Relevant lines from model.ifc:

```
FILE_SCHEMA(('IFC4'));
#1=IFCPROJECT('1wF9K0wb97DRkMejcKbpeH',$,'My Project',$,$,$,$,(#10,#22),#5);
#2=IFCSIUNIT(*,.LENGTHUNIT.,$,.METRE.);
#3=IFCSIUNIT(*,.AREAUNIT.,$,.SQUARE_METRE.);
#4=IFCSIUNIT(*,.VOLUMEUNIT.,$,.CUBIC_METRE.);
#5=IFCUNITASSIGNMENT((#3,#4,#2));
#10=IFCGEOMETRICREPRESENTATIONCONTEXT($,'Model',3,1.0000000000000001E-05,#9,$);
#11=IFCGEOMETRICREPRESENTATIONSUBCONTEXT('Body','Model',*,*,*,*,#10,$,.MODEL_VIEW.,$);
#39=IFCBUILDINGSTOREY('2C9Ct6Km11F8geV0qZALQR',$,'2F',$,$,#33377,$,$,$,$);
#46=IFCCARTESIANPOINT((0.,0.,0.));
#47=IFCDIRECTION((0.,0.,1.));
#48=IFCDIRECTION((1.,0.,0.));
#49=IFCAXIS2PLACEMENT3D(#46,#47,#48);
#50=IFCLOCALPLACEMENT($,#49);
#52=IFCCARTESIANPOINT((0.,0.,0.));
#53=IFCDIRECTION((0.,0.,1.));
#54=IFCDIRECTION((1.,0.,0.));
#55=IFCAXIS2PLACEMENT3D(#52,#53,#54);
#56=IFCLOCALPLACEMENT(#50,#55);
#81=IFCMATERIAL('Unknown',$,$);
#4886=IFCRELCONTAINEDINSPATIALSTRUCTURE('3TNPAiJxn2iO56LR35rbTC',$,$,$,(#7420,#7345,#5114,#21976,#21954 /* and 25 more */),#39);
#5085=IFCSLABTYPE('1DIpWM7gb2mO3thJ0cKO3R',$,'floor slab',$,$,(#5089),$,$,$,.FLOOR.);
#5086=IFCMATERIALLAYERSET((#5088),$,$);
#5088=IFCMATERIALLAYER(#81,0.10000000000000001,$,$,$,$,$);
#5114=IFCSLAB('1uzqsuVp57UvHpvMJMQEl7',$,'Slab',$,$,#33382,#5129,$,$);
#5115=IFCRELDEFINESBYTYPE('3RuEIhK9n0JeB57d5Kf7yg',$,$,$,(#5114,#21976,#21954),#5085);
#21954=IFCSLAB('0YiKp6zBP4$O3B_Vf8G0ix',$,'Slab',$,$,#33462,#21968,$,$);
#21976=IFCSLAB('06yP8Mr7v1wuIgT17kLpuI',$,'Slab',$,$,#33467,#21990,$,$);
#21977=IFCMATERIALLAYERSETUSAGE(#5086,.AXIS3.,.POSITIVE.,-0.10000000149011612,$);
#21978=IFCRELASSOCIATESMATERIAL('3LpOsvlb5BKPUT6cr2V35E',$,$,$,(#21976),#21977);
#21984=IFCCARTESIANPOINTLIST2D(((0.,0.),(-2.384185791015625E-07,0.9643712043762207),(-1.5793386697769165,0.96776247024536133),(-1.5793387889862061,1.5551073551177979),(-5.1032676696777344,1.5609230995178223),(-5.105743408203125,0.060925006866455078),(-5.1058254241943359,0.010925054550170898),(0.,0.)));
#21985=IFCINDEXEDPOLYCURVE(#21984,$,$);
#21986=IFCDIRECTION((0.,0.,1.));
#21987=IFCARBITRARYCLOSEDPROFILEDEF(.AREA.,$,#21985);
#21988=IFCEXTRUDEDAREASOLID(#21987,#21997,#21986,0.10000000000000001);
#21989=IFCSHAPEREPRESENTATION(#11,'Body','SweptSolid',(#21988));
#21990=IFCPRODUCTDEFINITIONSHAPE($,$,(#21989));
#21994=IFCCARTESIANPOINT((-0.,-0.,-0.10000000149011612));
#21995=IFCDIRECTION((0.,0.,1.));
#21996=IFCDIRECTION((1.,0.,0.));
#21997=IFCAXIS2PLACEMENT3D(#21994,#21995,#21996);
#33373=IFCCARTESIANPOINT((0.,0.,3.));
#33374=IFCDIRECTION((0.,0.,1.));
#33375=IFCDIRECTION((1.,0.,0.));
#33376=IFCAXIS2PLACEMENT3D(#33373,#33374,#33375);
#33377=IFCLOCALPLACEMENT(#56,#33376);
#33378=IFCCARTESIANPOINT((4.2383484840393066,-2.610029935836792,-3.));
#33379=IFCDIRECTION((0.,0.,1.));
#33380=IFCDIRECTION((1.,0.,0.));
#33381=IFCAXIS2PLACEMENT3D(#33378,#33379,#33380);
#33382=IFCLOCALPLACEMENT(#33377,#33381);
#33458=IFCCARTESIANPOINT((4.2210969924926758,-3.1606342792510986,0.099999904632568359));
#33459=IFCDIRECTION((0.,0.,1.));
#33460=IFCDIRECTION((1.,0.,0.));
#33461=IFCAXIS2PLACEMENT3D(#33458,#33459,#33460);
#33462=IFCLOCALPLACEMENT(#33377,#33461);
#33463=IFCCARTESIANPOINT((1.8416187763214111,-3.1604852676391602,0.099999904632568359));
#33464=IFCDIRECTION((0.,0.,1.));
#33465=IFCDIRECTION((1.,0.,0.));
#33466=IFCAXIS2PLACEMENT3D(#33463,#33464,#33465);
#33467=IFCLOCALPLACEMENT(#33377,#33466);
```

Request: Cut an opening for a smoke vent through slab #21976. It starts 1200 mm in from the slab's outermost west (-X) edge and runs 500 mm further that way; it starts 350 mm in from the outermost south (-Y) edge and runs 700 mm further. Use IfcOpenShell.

```python
import numpy as np
import ifcopenshell
import ifcopenshell.api.feature
import ifcopenshell.api.geometry
import ifcopenshell.api.root
import ifcopenshell.geom
import ifcopenshell.util.placement
import ifcopenshell.util.representation
import ifcopenshell.util.shape
import ifcopenshell.util.unit

model = ifcopenshell.open("model.ifc")
unit_scale = ifcopenshell.util.unit.calculate_unit_scale(model)
settings = ifcopenshell.geom.settings()


def volume(element):
    """Net volume in cubic metres, openings subtracted."""
    shape = ifcopenshell.geom.create_shape(settings, element)
    return ifcopenshell.util.shape.get_volume(shape.geometry)


slab = model.by_guid("06yP8Mr7v1wuIgT17kLpuI")
before = volume(slab)

# Extent in the slab's own axes, in metres. The edges named are its -X and -Y sides.
slab_shape = ifcopenshell.geom.create_shape(settings, slab)
vertices = ifcopenshell.util.shape.get_vertices(slab_shape.geometry)
x_min, y_min, bottom = vertices.min(axis=0)
top = vertices[:, 2].max()

opening = ifcopenshell.api.root.create_entity(model, ifc_class="IfcOpeningElement", name="Smoke vent opening", predefined_type="OPENING")
context = ifcopenshell.util.representation.get_context(model, "Model", "Body", "MODEL_VIEW")
width, depth = 0.5, 0.7
outline = [(0.0, 0.0), (width, 0.0), (width, depth), (0.0, depth), (0.0, 0.0)]
# Overshoot both faces by 50 mm so the cut is clean.
shape = ifcopenshell.api.geometry.add_slab_representation(
    model, context=context, depth=top - bottom + 0.1, polyline=outline
)
ifcopenshell.api.geometry.assign_representation(model, product=opening, representation=shape)

matrix = ifcopenshell.util.placement.get_local_placement(slab.ObjectPlacement)
matrix[:, 3] = matrix @ np.append(np.array([x_min + 1.2, y_min + 0.35, bottom - 0.05]) / unit_scale, 1.0)
ifcopenshell.api.geometry.edit_object_placement(model, product=opening, matrix=matrix, is_si=False)
ifcopenshell.api.feature.add_feature(model, feature=opening, element=slab)

after = volume(slab)

print(f"slab volume {before:.3f} -> {after:.3f} m3")

model.write("model_edited.ifc")
```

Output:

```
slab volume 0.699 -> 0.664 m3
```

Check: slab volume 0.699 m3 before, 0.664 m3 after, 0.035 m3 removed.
